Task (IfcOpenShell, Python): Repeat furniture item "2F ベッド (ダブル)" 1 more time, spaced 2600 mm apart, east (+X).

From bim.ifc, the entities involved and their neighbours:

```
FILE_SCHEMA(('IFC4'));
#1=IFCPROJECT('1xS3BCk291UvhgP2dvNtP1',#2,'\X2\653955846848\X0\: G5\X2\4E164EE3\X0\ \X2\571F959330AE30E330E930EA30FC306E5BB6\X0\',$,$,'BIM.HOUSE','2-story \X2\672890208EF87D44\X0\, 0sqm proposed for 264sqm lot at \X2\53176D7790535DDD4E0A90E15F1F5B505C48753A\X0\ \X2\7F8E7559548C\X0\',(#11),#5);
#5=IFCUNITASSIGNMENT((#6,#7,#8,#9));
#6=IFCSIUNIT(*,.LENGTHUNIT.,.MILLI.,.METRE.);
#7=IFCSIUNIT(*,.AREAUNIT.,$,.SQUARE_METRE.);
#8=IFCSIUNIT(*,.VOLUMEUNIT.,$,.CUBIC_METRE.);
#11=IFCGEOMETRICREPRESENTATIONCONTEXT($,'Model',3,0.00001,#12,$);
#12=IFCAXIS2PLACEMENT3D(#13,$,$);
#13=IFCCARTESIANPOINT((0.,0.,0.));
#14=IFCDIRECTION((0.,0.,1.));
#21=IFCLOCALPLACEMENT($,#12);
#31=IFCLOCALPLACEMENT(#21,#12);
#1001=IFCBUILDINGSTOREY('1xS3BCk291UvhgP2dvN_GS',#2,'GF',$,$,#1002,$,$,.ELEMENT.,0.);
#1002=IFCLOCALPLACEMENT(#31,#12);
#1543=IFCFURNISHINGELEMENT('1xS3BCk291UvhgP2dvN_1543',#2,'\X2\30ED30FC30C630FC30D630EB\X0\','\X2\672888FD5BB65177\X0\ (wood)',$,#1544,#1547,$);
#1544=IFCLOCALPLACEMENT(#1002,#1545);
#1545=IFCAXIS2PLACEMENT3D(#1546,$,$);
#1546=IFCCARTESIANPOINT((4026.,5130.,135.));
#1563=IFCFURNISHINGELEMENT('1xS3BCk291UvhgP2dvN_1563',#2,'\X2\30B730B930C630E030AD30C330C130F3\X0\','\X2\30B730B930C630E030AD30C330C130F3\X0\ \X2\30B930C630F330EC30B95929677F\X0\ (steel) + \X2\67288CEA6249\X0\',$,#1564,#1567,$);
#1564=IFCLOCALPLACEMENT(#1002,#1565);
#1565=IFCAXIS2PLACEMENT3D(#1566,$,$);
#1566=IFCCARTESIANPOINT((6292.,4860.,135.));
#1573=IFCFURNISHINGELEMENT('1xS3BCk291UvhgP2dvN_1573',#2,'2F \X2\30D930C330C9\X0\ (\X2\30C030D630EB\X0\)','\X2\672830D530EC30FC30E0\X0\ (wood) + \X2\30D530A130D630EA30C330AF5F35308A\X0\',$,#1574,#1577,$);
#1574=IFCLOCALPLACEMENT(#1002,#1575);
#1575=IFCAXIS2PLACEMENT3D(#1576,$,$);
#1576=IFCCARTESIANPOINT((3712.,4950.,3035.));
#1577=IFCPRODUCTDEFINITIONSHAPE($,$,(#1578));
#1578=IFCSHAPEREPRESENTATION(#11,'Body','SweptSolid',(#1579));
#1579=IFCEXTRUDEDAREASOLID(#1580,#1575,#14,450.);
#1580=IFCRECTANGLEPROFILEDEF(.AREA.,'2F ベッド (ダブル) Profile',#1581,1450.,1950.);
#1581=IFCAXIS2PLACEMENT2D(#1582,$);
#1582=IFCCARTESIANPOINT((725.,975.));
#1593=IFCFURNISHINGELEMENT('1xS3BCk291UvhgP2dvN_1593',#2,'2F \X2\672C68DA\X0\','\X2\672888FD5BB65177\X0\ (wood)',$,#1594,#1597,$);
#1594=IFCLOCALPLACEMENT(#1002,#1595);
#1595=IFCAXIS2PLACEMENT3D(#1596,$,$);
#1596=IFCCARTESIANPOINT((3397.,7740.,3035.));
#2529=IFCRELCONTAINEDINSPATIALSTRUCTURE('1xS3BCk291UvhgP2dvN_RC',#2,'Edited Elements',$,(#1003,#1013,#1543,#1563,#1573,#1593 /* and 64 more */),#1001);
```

```python
import numpy as np
import ifcopenshell
import ifcopenshell.api.geometry
import ifcopenshell.api.root
import ifcopenshell.util.element
import ifcopenshell.util.placement

model = ifcopenshell.open("bim.ifc")


def reuse_history(source, copy):
    """copy_class also copies each property set's owner history, people and application; keep the originals."""
    for rel in copy.IsDefinedBy:
        if rel.is_a("IfcRelDefinesByProperties") and (history := rel.RelatingPropertyDefinition.OwnerHistory):
            rel.RelatingPropertyDefinition.OwnerHistory = source.OwnerHistory
            ifcopenshell.util.element.remove_deep2(model, history)


source = model.by_guid("1xS3BCk291UvhgP2dvN_1573")
base = ifcopenshell.util.placement.get_local_placement(source.ObjectPlacement)
step = np.array([1.0, 0.0, 0.0]) * 2600.0

for i in range(1, 2):
    copy = ifcopenshell.api.root.copy_class(model, product=source)
    copy.Representation = ifcopenshell.util.element.copy_deep(
        model, source.Representation, exclude=["IfcGeometricRepresentationContext", "IfcRepresentationMap"]
    )
    reuse_history(source, copy)
    matrix = base.copy()
    matrix[:3, 3] += i * step
    print("added at", matrix[:3, 3].round(3) + 0.0)
    ifcopenshell.api.geometry.edit_object_placement(model, product=copy, matrix=matrix, is_si=False)

model.write("bim_edited.ifc")
```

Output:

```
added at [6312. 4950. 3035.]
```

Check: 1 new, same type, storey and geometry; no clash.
